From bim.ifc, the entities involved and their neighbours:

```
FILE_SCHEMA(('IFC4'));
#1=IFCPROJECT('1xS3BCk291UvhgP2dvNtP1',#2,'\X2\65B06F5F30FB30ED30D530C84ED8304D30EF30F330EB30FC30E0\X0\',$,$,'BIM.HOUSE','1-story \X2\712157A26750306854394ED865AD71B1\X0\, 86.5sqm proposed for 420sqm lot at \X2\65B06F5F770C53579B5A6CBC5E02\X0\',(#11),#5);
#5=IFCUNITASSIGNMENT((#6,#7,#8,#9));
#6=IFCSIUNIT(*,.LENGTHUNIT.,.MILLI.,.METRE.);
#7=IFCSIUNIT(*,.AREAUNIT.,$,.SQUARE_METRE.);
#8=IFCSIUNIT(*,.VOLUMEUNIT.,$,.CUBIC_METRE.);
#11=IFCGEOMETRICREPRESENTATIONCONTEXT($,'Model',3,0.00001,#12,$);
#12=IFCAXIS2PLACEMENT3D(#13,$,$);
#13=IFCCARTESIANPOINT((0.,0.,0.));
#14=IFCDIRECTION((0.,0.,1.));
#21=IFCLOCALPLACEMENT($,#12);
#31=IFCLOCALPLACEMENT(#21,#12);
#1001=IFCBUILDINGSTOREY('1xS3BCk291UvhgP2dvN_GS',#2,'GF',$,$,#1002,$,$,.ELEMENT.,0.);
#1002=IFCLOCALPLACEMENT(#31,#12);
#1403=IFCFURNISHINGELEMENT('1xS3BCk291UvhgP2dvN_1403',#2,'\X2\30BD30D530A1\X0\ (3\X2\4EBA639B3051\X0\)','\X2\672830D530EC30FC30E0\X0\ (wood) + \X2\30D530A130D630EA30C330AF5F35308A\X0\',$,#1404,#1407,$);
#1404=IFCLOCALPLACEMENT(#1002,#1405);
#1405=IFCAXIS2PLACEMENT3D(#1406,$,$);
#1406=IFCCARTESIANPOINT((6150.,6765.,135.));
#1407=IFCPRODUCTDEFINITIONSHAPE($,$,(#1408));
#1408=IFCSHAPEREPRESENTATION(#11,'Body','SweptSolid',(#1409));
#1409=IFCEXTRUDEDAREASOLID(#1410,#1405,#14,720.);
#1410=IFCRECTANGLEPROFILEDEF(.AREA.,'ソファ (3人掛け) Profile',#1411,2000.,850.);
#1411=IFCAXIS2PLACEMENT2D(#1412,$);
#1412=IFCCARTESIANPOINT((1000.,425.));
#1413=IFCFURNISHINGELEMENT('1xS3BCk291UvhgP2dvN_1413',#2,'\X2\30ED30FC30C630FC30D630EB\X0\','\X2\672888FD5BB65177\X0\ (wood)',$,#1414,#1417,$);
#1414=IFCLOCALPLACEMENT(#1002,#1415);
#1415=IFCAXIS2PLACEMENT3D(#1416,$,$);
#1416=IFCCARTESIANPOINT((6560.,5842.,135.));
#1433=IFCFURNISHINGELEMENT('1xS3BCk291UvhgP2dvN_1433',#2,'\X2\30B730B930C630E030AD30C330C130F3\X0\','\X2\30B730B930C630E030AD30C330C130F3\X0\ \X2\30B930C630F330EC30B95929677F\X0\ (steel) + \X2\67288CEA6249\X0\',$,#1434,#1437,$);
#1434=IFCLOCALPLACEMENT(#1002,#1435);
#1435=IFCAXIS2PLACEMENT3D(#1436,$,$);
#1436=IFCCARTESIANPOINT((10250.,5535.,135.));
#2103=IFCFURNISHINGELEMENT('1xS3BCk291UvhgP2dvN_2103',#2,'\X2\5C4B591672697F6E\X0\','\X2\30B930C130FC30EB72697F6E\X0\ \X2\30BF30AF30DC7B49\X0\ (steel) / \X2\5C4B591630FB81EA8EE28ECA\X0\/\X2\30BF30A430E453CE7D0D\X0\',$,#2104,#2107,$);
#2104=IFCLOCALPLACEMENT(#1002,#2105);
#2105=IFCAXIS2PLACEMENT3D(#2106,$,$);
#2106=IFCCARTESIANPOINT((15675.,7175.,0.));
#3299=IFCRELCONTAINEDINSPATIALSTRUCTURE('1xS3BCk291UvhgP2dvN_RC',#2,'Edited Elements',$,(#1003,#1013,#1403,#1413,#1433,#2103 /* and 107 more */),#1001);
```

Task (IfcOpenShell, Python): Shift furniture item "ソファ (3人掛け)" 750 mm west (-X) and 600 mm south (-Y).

```python
import ifcopenshell
import ifcopenshell.api.geometry
import ifcopenshell.util.placement

model = ifcopenshell.open("bim.ifc")

item = model.by_guid("1xS3BCk291UvhgP2dvN_1403")
matrix = ifcopenshell.util.placement.get_local_placement(item.ObjectPlacement)
matrix[0, 3] -= 750.0
matrix[1, 3] -= 600.0
ifcopenshell.api.geometry.edit_object_placement(model, product=item, matrix=matrix, is_si=False)

print(ifcopenshell.util.placement.get_local_placement(item.ObjectPlacement).round(3) + 0.0)

model.write("bim_rev.ifc")
```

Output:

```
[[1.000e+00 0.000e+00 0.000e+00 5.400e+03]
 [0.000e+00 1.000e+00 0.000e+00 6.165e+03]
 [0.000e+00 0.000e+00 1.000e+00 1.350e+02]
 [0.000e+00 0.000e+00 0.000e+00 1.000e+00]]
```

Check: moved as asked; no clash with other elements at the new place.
